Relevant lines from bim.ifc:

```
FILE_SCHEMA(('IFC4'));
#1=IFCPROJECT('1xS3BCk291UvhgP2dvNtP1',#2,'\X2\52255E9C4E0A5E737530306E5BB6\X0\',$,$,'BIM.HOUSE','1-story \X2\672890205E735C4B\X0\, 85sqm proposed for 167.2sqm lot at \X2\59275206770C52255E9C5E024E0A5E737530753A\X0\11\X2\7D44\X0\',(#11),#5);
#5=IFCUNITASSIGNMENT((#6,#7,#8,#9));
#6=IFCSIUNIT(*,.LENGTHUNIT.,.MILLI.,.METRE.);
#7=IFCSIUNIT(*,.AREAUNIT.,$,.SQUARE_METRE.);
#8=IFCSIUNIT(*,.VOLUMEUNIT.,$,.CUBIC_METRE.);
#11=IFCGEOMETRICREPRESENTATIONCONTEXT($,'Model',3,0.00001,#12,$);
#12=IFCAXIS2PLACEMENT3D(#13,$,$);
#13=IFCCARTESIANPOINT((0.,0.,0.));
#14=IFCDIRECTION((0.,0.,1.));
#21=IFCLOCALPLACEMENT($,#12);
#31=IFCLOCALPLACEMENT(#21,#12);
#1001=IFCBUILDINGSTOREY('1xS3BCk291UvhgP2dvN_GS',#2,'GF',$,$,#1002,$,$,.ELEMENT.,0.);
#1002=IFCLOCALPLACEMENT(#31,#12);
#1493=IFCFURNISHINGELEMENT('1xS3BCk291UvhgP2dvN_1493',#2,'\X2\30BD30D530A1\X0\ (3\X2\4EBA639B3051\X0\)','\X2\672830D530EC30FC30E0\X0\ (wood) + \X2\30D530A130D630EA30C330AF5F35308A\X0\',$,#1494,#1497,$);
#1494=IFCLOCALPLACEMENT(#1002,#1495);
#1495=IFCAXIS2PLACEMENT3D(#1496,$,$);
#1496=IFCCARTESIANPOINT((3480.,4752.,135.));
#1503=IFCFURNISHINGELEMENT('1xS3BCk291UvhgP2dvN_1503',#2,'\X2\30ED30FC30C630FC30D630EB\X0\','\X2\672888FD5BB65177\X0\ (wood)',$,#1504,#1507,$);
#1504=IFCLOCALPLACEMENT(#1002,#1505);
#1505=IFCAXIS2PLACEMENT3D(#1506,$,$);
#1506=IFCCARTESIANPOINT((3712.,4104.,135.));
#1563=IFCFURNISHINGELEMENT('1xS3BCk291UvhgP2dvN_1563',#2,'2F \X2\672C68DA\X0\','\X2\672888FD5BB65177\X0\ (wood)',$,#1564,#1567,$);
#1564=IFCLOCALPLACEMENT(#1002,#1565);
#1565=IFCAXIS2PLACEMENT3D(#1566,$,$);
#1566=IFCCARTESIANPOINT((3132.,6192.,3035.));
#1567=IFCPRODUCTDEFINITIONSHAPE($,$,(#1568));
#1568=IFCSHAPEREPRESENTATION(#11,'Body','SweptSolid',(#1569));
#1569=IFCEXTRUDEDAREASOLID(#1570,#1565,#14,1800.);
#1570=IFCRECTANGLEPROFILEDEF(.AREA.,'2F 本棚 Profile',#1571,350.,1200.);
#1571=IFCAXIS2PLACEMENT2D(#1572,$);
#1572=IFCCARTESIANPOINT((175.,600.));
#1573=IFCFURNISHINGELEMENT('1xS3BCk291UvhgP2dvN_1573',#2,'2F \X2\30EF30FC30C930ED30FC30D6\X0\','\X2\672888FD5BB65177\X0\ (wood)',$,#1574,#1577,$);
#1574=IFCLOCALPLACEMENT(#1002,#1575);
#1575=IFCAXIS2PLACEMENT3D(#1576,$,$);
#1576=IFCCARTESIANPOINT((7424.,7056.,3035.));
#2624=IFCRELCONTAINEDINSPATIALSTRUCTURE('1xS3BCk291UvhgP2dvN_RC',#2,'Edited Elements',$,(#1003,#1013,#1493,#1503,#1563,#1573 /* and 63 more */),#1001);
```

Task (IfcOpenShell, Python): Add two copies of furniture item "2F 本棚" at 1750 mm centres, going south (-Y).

```python
import numpy as np
import ifcopenshell
import ifcopenshell.api.geometry
import ifcopenshell.api.root
import ifcopenshell.util.element
import ifcopenshell.util.placement
import ifcopenshell.util.unit

model = ifcopenshell.open("bim.ifc")
unit_scale = ifcopenshell.util.unit.calculate_unit_scale(model)


def reuse_history(source, copy):
    """copy_class also copies each property set's owner history, people and application; keep the originals."""
    for rel in copy.IsDefinedBy:
        if rel.is_a("IfcRelDefinesByProperties") and (history := rel.RelatingPropertyDefinition.OwnerHistory):
            rel.RelatingPropertyDefinition.OwnerHistory = source.OwnerHistory
            ifcopenshell.util.element.remove_deep2(model, history)


source = model.by_id(1563)
base = ifcopenshell.util.placement.get_local_placement(source.ObjectPlacement)
step = np.array([0.0, -1.0, 0.0]) * 1.75 / unit_scale

for i in range(1, 3):
    copy = ifcopenshell.api.root.copy_class(model, product=source)
    copy.Representation = ifcopenshell.util.element.copy_deep(
        model, source.Representation, exclude=["IfcGeometricRepresentationContext", "IfcRepresentationMap"]
    )
    reuse_history(source, copy)
    matrix = base.copy()
    matrix[:3, 3] += i * step
    print("added at", matrix[:3, 3].round(3) + 0.0)
    ifcopenshell.api.geometry.edit_object_placement(model, product=copy, matrix=matrix, is_si=False)

model.write("bim_v2.ifc")
```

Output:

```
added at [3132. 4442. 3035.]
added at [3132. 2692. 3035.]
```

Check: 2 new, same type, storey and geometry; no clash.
